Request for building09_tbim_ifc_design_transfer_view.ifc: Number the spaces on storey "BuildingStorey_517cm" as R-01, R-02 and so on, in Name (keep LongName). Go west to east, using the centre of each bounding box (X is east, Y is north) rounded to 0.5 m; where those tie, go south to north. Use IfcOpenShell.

First a look at what the model holds.

```python
import ifcopenshell
import ifcopenshell.util.element
import ifcopenshell.util.placement

model = ifcopenshell.open("building09_tbim_ifc_design_transfer_view.ifc")
print(model.schema)
storey = next(s for s in model.by_type("IfcBuildingStorey") if s.Name == "BuildingStorey_517cm")
spaces = [e for e in ifcopenshell.util.element.get_decomposition(storey) if e.is_a("IfcSpace")]
for e in sorted(spaces, key=lambda e: e.id()):
    origin = ifcopenshell.util.placement.get_local_placement(e.ObjectPlacement)[:3, 3]
    print(e.id(), e.Name, e.LongName, origin.round(2) + 0.0, sep=" | ")
```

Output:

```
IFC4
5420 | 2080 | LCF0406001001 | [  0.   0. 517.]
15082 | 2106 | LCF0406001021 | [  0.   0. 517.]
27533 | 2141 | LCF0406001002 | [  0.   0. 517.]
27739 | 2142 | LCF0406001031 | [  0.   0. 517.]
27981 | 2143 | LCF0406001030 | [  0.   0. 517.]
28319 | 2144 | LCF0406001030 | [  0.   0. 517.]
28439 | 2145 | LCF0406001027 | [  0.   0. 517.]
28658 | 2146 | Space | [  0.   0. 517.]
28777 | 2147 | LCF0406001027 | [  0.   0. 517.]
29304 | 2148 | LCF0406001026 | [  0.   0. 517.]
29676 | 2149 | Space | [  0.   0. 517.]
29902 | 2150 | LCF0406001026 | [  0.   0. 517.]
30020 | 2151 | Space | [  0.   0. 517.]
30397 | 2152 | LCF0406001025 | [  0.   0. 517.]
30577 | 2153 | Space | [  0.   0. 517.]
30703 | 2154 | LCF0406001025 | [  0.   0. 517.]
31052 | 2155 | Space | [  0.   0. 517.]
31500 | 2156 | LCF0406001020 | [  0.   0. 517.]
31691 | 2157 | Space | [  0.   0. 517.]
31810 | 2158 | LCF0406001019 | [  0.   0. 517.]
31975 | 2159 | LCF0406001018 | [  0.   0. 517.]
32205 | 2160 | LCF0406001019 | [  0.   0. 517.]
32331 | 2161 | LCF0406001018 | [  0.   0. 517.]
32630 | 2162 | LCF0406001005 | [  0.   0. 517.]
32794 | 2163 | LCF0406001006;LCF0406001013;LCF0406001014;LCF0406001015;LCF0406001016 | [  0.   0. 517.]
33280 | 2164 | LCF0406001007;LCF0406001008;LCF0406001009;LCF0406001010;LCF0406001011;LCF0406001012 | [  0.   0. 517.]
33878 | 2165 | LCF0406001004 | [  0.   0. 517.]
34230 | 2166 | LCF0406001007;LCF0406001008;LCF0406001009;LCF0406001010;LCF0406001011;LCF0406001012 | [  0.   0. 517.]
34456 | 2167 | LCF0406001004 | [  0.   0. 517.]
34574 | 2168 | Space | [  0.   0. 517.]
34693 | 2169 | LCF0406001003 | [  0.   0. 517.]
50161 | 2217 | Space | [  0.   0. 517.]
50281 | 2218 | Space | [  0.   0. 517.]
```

```python
import ifcopenshell
import ifcopenshell.geom
import ifcopenshell.util.element
import ifcopenshell.util.shape

model = ifcopenshell.open("building09_tbim_ifc_design_transfer_view.ifc")
settings = ifcopenshell.geom.settings()
settings.set("use-world-coords", True)


def centre(element):
    shape = ifcopenshell.geom.create_shape(settings, element)
    return ifcopenshell.util.shape.get_bbox_centroid(shape.geometry)


storey = next(s for s in model.by_type("IfcBuildingStorey") if s.Name == "BuildingStorey_517cm")
spaces = [e for e in ifcopenshell.util.element.get_decomposition(storey) if e.is_a("IfcSpace")]

# Insertion points can sit at a corner or the storey origin, so sort by the geometry (in metres).
centres = {e: centre(e) for e in spaces}
spaces.sort(key=lambda e: (round(centres[e][0] / 0.5), centres[e][1]))

for i, e in enumerate(spaces, start=1):
    number = f"R-{i:02d}"
    e.Name = number
    print(e.id(), number)

model.write("building09_tbim_ifc_design_transfer_view-out.ifc")
```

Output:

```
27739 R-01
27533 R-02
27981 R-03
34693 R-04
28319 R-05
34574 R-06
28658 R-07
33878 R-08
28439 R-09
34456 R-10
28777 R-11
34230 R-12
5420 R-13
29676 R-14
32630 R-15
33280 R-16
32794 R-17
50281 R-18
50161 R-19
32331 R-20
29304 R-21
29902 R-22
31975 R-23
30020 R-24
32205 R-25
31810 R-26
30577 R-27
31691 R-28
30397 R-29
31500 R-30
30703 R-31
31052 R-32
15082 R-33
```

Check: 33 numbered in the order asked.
